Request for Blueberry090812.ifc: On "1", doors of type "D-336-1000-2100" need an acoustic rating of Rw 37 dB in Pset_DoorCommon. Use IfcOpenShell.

First a look at what the model holds.

```python
import ifcopenshell
import ifcopenshell.util.element

model = ifcopenshell.open("Blueberry090812.ifc")
print(model.schema)
storey = next(s for s in model.by_type("IfcBuildingStorey") if s.Name == "1")
doors = [e for e in ifcopenshell.util.element.get_decomposition(storey) if e.is_a("IfcDoor")]
seen = {}
for e in doors:
    element_type = ifcopenshell.util.element.get_type(e)
    key = (element_type.Name if element_type != e and element_type else None, ifcopenshell.util.element.get_pset(e, "Pset_DoorCommon", "AcousticRating"))
    seen[key] = seen.get(key, 0) + 1
for (name, value), count in sorted(seen.items(), key=str):
    print(count, "x", name, "|", value)
```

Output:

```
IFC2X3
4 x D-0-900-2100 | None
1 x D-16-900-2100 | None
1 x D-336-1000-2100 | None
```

```python
import ifcopenshell
import ifcopenshell.api.pset
import ifcopenshell.util.element

model = ifcopenshell.open("Blueberry090812.ifc")

storey = next(s for s in model.by_type("IfcBuildingStorey") if s.Name == "1")
doors = [e for e in ifcopenshell.util.element.get_decomposition(storey) if e.is_a("IfcDoor")]

count = 0
for e in doors:
    element_type = ifcopenshell.util.element.get_type(e)
    if element_type in (None, e) or element_type.Name != "D-336-1000-2100":
        continue
    # add_pset returns the element's existing set when there is one.
    pset = ifcopenshell.api.pset.add_pset(model, product=e, name="Pset_DoorCommon")
    ifcopenshell.api.pset.edit_pset(model, pset=pset, properties={"AcousticRating": "Rw 37 dB"})
    count += 1

print(count, "doors updated")

model.write("Blueberry090812_rev.ifc")
```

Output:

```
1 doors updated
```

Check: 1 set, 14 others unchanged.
